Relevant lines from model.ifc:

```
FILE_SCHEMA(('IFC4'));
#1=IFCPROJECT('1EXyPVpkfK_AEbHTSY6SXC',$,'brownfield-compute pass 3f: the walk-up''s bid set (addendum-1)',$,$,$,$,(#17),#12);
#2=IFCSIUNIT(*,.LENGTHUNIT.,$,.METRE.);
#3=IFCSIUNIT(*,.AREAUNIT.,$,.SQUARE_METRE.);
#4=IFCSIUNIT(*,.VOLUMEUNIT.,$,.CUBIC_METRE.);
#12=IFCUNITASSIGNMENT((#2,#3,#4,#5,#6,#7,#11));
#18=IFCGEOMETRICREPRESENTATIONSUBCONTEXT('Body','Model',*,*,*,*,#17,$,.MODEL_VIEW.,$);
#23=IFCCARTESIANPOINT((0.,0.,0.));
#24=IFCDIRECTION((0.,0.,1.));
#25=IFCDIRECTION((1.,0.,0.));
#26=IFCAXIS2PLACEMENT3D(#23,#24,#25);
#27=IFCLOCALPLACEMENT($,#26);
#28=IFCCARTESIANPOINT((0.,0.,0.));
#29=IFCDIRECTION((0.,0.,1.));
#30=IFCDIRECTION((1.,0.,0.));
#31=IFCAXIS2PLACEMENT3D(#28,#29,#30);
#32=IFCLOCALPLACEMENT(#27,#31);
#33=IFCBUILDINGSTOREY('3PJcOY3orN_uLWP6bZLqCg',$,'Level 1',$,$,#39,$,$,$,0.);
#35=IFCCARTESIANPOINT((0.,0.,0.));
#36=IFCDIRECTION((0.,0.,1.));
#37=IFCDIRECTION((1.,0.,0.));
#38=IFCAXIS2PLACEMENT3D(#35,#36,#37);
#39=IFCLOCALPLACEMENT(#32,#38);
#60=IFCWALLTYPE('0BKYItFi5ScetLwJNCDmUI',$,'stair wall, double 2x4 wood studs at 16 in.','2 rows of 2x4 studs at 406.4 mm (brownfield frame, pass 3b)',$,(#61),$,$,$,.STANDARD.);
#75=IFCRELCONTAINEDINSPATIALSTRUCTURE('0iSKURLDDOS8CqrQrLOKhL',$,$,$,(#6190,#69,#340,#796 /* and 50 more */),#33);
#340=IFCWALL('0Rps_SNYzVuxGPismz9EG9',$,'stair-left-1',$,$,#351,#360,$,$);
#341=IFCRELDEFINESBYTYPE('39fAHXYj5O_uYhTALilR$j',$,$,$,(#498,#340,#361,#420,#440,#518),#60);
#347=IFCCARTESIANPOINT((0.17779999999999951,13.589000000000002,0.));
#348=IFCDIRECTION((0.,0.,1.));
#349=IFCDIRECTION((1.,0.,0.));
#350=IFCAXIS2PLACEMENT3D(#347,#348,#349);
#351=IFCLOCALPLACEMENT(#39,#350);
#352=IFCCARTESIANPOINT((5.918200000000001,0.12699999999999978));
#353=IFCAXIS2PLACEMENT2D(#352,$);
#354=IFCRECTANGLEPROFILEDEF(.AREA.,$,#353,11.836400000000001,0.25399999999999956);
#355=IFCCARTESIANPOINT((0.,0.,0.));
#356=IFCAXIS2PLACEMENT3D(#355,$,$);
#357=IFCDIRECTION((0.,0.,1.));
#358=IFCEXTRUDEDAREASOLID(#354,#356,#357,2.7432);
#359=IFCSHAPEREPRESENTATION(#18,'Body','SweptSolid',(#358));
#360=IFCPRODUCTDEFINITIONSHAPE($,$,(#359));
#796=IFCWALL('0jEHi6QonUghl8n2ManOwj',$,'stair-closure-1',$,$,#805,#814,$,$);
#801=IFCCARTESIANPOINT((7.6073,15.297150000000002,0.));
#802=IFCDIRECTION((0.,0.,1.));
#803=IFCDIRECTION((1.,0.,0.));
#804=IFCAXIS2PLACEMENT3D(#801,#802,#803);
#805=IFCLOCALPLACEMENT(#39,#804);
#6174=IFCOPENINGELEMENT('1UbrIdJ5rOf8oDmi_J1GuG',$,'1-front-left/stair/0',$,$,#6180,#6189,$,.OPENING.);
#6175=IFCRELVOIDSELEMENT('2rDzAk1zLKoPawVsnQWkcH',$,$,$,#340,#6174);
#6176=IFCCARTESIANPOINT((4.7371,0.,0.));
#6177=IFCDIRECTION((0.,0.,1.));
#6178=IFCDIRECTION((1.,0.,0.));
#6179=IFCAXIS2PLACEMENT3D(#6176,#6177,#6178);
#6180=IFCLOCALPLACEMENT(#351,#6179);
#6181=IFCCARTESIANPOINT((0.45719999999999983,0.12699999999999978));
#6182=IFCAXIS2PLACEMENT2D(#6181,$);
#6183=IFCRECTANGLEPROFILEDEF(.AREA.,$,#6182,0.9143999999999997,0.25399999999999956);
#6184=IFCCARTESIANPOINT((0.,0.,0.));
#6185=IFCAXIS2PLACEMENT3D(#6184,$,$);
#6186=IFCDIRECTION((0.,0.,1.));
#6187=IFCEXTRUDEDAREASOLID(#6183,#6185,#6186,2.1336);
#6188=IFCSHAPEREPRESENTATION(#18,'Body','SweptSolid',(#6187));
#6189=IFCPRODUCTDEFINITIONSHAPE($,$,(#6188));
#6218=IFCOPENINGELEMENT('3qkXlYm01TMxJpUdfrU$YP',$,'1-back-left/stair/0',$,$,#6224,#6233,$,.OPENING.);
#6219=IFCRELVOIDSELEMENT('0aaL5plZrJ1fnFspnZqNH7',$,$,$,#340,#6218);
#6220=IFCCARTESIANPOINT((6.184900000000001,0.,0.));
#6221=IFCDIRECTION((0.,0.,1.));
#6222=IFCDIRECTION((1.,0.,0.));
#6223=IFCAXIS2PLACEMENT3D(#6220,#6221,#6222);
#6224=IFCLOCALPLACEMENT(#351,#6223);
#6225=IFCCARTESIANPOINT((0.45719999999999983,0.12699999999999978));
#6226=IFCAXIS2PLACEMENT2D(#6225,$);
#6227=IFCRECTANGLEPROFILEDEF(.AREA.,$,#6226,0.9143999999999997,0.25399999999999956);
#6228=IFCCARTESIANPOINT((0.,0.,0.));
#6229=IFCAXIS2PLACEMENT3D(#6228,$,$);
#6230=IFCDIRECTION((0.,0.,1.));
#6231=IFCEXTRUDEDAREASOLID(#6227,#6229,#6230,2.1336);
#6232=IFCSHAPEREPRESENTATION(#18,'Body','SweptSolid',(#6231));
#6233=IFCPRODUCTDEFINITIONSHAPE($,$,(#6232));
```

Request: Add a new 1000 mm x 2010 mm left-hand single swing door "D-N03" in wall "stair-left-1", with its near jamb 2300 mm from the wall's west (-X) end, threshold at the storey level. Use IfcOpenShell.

```python
import numpy as np
import ifcopenshell
import ifcopenshell.api.feature
import ifcopenshell.api.geometry
import ifcopenshell.api.root
import ifcopenshell.api.spatial
import ifcopenshell.geom
import ifcopenshell.util.element
import ifcopenshell.util.placement
import ifcopenshell.util.representation
import ifcopenshell.util.shape
import ifcopenshell.util.unit

model = ifcopenshell.open("model.ifc")
unit_scale = ifcopenshell.util.unit.calculate_unit_scale(model)
settings = ifcopenshell.geom.settings()


def volume(element):
    """Net volume in cubic metres, openings subtracted."""
    shape = ifcopenshell.geom.create_shape(settings, element)
    return ifcopenshell.util.shape.get_volume(shape.geometry)


wall = model.by_id(340)
storey = ifcopenshell.util.element.get_container(wall, ifc_class="IfcBuildingStorey")
context = ifcopenshell.util.representation.get_context(model, "Model", "Body", "MODEL_VIEW")
before = volume(wall)

width, height, from_end, sill = 1, 2.01, 2.3, 0.0  # metres

# The wall runs along its own X axis, and the end named is its -X end.
wall_shape = ifcopenshell.geom.create_shape(settings, wall)
x, y, z = ifcopenshell.util.shape.get_vertices(wall_shape.geometry).T
start = x.min() + from_end
face, thickness = float(y.min()), float(y.max() - y.min())
wall_matrix = ifcopenshell.util.placement.get_local_placement(wall.ObjectPlacement)
level = ifcopenshell.util.placement.get_local_placement(storey.ObjectPlacement)[2, 3]


def in_wall(x, y):
    """Placement at x, y metres in the wall's axes, at sill height."""
    matrix = wall_matrix.copy()
    matrix[:, 3] = wall_matrix @ np.array([x / unit_scale, y / unit_scale, 0.0, 1.0])
    matrix[2, 3] = level + sill / unit_scale
    return matrix


# Opening: a box that overshoots both wall faces by 50 mm.
opening = ifcopenshell.api.root.create_entity(model, ifc_class="IfcOpeningElement", predefined_type="OPENING")
box = ifcopenshell.api.geometry.add_wall_representation(
    model, context=context, length=width, height=height, thickness=thickness + 0.1
)
ifcopenshell.api.geometry.assign_representation(model, product=opening, representation=box)
ifcopenshell.api.geometry.edit_object_placement(model, product=opening, matrix=in_wall(start, face - 0.05), is_si=False)
ifcopenshell.api.feature.add_feature(model, feature=opening, element=wall)

door = ifcopenshell.api.root.create_entity(model, ifc_class="IfcDoor", name="D-N03", predefined_type="DOOR")
door.OverallWidth, door.OverallHeight = width / unit_scale, height / unit_scale
door.OperationType = "SINGLE_SWING_LEFT"
body = ifcopenshell.api.geometry.add_door_representation(
    model,
    context=context,
    overall_width=door.OverallWidth,
    overall_height=door.OverallHeight,
    operation_type="SINGLE_SWING_LEFT",
    lining_properties={"LiningDepth": thickness / unit_scale, "ThresholdDepth": thickness / unit_scale},
)
ifcopenshell.api.geometry.assign_representation(model, product=door, representation=body)
ifcopenshell.api.spatial.assign_container(model, products=[door], relating_structure=storey)
ifcopenshell.api.feature.add_filling(model, opening=opening, element=door)

# The lining spans the wall, so the door starts at the wall face.
ifcopenshell.api.geometry.edit_object_placement(model, product=door, matrix=in_wall(start, face), is_si=False)

after = volume(wall)

print(f"wall volume {before:.3f} -> {after:.3f} m3")

model.write("model_v2.ifc")
```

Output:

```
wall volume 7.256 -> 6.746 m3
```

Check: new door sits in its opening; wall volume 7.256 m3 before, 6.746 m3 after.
